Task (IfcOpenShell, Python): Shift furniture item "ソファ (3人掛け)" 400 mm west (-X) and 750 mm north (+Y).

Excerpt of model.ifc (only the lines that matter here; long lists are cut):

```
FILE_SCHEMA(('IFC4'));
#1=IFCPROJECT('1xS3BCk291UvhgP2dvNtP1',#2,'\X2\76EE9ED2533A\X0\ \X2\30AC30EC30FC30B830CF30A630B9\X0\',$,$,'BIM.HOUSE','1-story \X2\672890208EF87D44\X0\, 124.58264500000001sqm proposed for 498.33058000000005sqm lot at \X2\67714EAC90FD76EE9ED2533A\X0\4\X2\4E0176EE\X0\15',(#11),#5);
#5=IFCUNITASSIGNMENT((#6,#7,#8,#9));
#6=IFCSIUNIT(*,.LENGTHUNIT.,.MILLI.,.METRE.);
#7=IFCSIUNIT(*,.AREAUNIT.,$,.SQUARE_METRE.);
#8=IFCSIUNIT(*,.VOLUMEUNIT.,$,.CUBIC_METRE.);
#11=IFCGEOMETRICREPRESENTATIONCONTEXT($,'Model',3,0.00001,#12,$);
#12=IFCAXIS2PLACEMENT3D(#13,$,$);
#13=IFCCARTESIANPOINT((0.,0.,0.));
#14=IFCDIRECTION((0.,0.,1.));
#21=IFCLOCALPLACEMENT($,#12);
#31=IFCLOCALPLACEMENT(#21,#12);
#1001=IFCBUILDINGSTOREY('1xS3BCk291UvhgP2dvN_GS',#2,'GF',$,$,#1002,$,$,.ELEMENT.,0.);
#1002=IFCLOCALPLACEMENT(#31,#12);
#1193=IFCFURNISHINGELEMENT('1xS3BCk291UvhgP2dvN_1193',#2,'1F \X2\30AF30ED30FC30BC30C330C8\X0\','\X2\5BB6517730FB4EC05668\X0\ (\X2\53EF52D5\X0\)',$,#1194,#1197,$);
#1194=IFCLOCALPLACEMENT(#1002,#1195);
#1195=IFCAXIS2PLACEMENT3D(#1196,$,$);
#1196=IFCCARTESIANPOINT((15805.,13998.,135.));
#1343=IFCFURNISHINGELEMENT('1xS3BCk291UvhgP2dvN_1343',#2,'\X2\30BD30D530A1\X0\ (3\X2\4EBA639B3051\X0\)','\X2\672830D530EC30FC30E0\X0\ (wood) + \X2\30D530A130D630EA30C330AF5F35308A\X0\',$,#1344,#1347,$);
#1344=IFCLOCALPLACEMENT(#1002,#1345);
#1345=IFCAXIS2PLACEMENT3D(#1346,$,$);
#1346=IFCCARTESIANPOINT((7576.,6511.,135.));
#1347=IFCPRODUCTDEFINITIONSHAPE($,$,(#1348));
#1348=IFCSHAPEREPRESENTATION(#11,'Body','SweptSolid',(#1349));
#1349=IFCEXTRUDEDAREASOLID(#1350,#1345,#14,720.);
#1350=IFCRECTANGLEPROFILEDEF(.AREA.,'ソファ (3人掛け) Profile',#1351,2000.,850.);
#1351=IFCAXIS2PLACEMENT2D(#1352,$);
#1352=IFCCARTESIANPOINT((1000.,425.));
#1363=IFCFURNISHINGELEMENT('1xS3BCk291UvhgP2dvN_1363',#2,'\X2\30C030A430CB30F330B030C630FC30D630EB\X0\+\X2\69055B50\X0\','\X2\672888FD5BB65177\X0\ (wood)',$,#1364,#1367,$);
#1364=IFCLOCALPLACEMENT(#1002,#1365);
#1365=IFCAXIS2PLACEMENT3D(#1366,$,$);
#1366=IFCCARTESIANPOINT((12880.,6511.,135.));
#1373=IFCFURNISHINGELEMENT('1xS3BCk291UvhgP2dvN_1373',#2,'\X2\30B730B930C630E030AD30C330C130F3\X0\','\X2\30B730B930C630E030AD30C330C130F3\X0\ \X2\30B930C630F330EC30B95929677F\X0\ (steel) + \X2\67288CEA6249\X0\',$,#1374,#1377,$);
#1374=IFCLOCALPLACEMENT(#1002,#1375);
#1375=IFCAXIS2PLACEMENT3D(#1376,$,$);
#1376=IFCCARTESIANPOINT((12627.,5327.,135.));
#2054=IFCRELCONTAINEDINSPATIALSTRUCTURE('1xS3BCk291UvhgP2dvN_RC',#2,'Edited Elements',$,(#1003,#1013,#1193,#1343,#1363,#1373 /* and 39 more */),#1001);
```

```python
import ifcopenshell
import ifcopenshell.api.geometry
import ifcopenshell.util.placement

model = ifcopenshell.open("model.ifc")

item = model.by_guid("1xS3BCk291UvhgP2dvN_1343")
matrix = ifcopenshell.util.placement.get_local_placement(item.ObjectPlacement)
matrix[0, 3] -= 400.0
matrix[1, 3] += 750.0
ifcopenshell.api.geometry.edit_object_placement(model, product=item, matrix=matrix, is_si=False)

print(ifcopenshell.util.placement.get_local_placement(item.ObjectPlacement).round(3) + 0.0)

model.write("model_edited.ifc")
```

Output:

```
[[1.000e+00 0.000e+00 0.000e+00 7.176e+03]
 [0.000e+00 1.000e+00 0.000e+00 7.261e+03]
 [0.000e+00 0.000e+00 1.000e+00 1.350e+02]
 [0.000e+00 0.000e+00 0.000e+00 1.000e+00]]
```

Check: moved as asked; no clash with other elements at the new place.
